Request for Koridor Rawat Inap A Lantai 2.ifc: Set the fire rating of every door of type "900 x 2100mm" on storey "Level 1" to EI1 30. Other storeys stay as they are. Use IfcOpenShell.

First a look at what the model holds.

```python
import ifcopenshell
import ifcopenshell.util.element

model = ifcopenshell.open("Koridor Rawat Inap A Lantai 2.ifc")
print(model.schema)
storey = next(s for s in model.by_type("IfcBuildingStorey") if s.Name == "Level 1")
doors = [e for e in ifcopenshell.util.element.get_decomposition(storey) if e.is_a("IfcDoor")]
seen = {}
for e in doors:
    element_type = ifcopenshell.util.element.get_type(e)
    key = (element_type.Name if element_type != e and element_type else None, ifcopenshell.util.element.get_pset(e, "Pset_DoorCommon", "FireRating"))
    seen[key] = seen.get(key, 0) + 1
for (name, value), count in sorted(seen.items(), key=str):
    print(count, "x", name, "|", value)
```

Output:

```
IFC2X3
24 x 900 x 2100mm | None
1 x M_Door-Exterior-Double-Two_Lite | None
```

```python
import ifcopenshell
import ifcopenshell.api.pset
import ifcopenshell.util.element

model = ifcopenshell.open("Koridor Rawat Inap A Lantai 2.ifc")

storey = next(s for s in model.by_type("IfcBuildingStorey") if s.Name == "Level 1")
doors = [e for e in ifcopenshell.util.element.get_decomposition(storey) if e.is_a("IfcDoor")]

count = 0
for e in doors:
    element_type = ifcopenshell.util.element.get_type(e)
    if element_type in (None, e) or element_type.Name != "900 x 2100mm":
        continue
    # add_pset returns the element's existing set when there is one.
    pset = ifcopenshell.api.pset.add_pset(model, product=e, name="Pset_DoorCommon")
    ifcopenshell.api.pset.edit_pset(model, pset=pset, properties={"FireRating": "EI1 30"})
    count += 1

print(count, "doors updated")

model.write("Koridor Rawat Inap A Lantai 2_updated.ifc")
```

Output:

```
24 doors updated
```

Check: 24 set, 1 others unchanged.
